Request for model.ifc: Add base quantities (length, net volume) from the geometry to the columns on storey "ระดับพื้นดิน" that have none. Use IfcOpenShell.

First a look at what the model holds.

```python
import ifcopenshell
import ifcopenshell.util.element
import ifcopenshell.util.unit

model = ifcopenshell.open("model.ifc")
print(model.schema)
for unit_type in ("LENGTHUNIT", "AREAUNIT", "VOLUMEUNIT"):
    print(unit_type, ifcopenshell.util.unit.calculate_unit_scale(model, unit_type))
storey = next(s for s in model.by_type("IfcBuildingStorey") if s.Name == "ระดับพื้นดิน")
columns = [e for e in ifcopenshell.util.element.get_decomposition(storey) if e.is_a("IfcColumn")]
for e in sorted(columns, key=lambda e: e.id()):
    print(e.id(), e.is_a(), e.Name, list(ifcopenshell.util.element.get_psets(e, qtos_only=True)), sep=" | ")
```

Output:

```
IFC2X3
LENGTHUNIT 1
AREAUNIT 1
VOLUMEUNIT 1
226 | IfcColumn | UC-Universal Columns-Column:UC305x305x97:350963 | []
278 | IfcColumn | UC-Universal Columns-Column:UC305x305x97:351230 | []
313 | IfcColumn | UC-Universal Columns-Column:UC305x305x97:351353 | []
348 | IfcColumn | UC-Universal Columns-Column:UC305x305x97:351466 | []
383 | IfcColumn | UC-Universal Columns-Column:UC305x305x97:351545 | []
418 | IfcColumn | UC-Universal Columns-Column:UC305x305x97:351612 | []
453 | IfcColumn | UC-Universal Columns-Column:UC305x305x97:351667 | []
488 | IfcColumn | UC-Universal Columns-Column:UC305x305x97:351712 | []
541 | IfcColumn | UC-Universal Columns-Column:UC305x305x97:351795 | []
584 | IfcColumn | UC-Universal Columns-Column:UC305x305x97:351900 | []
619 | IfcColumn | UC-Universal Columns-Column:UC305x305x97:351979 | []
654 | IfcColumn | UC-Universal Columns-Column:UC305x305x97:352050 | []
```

```python
import ifcopenshell
import ifcopenshell.api.pset
import ifcopenshell.geom
import ifcopenshell.util.element
import ifcopenshell.util.shape
import ifcopenshell.util.unit

model = ifcopenshell.open("model.ifc")
unit_scale = ifcopenshell.util.unit.calculate_unit_scale(model)
volume_scale = ifcopenshell.util.unit.calculate_unit_scale(model, "VOLUMEUNIT")
settings = ifcopenshell.geom.settings()

storey = next(s for s in model.by_type("IfcBuildingStorey") if s.Name == "ระดับพื้นดิน")
columns = [e for e in ifcopenshell.util.element.get_decomposition(storey) if e.is_a("IfcColumn")]

for e in sorted(columns, key=lambda e: e.id()):
    if ifcopenshell.util.element.get_psets(e, qtos_only=True, should_inherit=False):
        continue
    # Geometry comes back in metres, in the element's own axes.
    shape = ifcopenshell.geom.create_shape(settings, e)
    values = {
        "Length": ifcopenshell.util.shape.get_z(shape.geometry) / unit_scale,
        "NetVolume": ifcopenshell.util.shape.get_volume(shape.geometry) / volume_scale,
    }
    qto = ifcopenshell.api.pset.add_qto(model, product=e, name="BaseQuantities")
    ifcopenshell.api.pset.edit_qto(model, qto=qto, properties=values)
    print(e.id(), {k: round(v, 3) for k, v in values.items()})

model.write("model_updated.ifc")
```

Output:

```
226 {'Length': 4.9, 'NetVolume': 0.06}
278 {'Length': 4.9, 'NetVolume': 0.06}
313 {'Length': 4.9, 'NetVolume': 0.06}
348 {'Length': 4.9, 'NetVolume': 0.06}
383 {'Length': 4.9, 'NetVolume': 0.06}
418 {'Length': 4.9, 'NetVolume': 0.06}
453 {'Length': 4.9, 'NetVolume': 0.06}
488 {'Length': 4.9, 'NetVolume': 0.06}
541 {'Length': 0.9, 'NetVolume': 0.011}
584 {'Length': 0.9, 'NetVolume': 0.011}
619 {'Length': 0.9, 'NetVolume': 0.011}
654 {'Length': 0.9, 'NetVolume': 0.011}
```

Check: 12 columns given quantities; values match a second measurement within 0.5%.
